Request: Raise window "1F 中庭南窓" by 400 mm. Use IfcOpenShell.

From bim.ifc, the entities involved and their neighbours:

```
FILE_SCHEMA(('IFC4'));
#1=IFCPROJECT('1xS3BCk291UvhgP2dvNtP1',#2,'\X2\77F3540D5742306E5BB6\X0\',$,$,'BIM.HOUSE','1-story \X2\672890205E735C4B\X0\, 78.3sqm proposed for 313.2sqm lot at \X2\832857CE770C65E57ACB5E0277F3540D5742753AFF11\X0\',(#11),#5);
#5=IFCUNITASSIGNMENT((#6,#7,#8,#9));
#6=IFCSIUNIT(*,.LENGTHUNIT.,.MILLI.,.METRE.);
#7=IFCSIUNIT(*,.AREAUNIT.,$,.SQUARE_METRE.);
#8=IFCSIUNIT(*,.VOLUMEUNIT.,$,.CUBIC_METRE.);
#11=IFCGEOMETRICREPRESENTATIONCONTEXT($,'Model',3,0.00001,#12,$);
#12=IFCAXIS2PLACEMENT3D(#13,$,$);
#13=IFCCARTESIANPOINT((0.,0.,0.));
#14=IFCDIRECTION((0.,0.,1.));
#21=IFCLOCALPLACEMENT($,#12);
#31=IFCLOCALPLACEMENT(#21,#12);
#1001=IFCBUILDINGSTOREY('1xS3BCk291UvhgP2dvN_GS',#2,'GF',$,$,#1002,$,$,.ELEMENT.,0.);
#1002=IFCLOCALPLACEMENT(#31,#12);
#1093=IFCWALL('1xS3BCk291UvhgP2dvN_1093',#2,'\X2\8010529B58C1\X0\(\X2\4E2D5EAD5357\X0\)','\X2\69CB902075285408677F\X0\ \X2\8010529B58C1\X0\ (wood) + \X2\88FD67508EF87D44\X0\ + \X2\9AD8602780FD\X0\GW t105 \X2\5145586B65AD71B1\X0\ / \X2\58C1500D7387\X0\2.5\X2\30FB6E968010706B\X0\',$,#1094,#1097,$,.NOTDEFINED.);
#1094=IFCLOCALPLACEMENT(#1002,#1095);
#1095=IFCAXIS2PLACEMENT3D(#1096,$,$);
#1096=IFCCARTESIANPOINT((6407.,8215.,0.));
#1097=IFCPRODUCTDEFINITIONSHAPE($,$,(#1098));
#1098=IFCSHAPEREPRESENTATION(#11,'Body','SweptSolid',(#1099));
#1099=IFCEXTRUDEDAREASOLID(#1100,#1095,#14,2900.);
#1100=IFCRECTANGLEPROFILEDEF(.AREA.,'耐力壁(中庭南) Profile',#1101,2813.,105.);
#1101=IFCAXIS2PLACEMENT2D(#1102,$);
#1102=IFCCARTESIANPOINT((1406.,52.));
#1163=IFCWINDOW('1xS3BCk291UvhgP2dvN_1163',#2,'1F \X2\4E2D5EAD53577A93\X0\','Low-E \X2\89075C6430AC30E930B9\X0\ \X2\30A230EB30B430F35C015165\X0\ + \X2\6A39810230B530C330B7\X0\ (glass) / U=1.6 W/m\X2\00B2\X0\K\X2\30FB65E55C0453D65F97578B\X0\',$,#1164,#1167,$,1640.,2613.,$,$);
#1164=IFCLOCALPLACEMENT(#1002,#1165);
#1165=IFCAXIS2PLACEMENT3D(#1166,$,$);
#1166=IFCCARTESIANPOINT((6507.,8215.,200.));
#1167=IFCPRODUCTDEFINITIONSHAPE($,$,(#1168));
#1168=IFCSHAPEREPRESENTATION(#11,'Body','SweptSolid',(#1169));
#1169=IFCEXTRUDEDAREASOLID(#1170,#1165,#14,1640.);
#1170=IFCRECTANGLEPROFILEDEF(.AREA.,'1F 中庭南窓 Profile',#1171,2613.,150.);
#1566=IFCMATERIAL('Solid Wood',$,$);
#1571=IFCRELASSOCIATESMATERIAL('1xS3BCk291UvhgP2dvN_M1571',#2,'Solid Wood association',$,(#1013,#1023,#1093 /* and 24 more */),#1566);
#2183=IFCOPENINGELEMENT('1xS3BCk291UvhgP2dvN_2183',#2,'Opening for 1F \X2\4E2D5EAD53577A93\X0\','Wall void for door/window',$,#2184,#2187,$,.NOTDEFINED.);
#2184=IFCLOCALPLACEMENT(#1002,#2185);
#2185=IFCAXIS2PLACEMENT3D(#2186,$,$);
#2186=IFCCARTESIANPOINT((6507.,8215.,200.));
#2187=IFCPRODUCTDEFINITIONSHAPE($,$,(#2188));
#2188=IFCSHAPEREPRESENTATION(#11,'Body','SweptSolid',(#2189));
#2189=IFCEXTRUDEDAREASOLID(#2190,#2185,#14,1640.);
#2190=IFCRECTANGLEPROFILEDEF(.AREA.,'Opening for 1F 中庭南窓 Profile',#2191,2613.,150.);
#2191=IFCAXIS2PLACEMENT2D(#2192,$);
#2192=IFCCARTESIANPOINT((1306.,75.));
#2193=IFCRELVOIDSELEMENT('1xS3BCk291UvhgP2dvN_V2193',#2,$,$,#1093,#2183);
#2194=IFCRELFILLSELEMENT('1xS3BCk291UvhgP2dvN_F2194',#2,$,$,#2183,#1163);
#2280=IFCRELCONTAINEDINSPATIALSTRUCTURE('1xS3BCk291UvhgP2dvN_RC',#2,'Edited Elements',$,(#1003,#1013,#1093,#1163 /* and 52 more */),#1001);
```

```python
import numpy as np
import ifcopenshell
import ifcopenshell.api.geometry
import ifcopenshell.util.placement
import ifcopenshell.util.unit

model = ifcopenshell.open("bim.ifc")
unit_scale = ifcopenshell.util.unit.calculate_unit_scale(model)

window = model.by_guid("1xS3BCk291UvhgP2dvN_1163")
opening = window.FillsVoids[0].RelatingOpeningElement
dz = 0.4 / unit_scale

shift = np.array([0.0, 0.0, dz])
# The window is not placed relative to its opening, so move both.
for product in (opening, window):
    matrix = ifcopenshell.util.placement.get_local_placement(product.ObjectPlacement)
    matrix[:3, 3] += shift
    ifcopenshell.api.geometry.edit_object_placement(model, product=product, matrix=matrix, is_si=False)

print(f"moved by {dz * unit_scale:+.3f} m")

model.write("bim_rev.ifc")
```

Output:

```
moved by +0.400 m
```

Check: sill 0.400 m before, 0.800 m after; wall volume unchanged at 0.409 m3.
